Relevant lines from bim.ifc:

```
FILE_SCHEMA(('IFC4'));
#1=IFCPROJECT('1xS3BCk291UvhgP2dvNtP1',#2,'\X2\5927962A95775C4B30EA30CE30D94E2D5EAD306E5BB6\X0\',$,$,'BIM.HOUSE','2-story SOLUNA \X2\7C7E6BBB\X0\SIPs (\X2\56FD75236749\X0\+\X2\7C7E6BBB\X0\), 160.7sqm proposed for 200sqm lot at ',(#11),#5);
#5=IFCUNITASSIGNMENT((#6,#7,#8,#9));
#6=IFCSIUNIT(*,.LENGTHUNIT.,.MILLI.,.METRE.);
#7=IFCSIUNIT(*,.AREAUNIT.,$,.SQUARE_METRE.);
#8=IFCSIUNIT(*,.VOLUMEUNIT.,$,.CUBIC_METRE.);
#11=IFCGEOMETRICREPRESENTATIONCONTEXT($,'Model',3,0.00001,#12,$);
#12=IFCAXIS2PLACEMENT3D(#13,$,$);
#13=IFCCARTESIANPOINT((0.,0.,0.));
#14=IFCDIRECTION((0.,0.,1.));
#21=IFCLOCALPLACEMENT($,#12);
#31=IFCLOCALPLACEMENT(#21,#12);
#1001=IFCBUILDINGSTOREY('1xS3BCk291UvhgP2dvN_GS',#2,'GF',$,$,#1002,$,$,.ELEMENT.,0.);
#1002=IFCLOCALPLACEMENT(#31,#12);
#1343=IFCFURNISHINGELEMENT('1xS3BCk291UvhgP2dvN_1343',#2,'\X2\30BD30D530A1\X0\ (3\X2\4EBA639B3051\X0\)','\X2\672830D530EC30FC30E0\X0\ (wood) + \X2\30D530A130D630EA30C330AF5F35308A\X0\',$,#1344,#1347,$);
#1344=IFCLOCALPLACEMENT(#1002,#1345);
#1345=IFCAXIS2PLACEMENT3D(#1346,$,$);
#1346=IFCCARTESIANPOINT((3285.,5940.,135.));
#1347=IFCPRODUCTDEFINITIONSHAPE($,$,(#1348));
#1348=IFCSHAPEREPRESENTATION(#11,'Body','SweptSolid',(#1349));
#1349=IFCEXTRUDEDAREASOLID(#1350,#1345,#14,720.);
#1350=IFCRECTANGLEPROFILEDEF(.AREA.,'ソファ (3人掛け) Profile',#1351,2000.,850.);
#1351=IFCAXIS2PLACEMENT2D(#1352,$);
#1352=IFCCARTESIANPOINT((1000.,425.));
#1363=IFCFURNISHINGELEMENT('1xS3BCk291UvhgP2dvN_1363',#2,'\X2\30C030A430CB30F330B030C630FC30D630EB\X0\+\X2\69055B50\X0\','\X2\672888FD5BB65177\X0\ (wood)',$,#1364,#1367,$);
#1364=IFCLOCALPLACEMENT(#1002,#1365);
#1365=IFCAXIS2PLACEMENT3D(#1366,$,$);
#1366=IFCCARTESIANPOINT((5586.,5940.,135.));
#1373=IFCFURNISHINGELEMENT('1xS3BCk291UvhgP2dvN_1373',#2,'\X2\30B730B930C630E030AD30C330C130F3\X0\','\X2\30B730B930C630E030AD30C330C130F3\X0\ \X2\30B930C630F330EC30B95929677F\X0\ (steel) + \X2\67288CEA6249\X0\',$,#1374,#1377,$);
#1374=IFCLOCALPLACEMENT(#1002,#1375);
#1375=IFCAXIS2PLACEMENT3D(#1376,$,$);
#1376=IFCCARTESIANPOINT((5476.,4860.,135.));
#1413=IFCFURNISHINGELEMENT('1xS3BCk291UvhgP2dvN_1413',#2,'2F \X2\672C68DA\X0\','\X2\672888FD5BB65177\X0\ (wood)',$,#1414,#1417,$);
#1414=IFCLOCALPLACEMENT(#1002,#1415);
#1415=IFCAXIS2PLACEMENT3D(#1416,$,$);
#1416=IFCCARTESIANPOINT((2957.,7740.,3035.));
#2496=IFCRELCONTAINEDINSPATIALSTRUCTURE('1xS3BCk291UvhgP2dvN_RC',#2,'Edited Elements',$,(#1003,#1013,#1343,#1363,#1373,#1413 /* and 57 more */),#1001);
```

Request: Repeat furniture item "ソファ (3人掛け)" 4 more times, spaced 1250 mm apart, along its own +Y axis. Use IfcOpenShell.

```python
import ifcopenshell
import ifcopenshell.api.geometry
import ifcopenshell.api.root
import ifcopenshell.util.element
import ifcopenshell.util.placement

model = ifcopenshell.open("bim.ifc")


def reuse_history(source, copy):
    """copy_class also copies each property set's owner history, people and application; keep the originals."""
    for rel in copy.IsDefinedBy:
        if rel.is_a("IfcRelDefinesByProperties") and (history := rel.RelatingPropertyDefinition.OwnerHistory):
            rel.RelatingPropertyDefinition.OwnerHistory = source.OwnerHistory
            ifcopenshell.util.element.remove_deep2(model, history)


source = model.by_guid("1xS3BCk291UvhgP2dvN_1343")
base = ifcopenshell.util.placement.get_local_placement(source.ObjectPlacement)
step = base[:3, 1] * 1250.0

for i in range(1, 5):
    copy = ifcopenshell.api.root.copy_class(model, product=source)
    copy.Representation = ifcopenshell.util.element.copy_deep(
        model, source.Representation, exclude=["IfcGeometricRepresentationContext", "IfcRepresentationMap"]
    )
    reuse_history(source, copy)
    matrix = base.copy()
    matrix[:3, 3] += i * step
    print("added at", matrix[:3, 3].round(3) + 0.0)
    ifcopenshell.api.geometry.edit_object_placement(model, product=copy, matrix=matrix, is_si=False)

model.write("bim-out.ifc")
```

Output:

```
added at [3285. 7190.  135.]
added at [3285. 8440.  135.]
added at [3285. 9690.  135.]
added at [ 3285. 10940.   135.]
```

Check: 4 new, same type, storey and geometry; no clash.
